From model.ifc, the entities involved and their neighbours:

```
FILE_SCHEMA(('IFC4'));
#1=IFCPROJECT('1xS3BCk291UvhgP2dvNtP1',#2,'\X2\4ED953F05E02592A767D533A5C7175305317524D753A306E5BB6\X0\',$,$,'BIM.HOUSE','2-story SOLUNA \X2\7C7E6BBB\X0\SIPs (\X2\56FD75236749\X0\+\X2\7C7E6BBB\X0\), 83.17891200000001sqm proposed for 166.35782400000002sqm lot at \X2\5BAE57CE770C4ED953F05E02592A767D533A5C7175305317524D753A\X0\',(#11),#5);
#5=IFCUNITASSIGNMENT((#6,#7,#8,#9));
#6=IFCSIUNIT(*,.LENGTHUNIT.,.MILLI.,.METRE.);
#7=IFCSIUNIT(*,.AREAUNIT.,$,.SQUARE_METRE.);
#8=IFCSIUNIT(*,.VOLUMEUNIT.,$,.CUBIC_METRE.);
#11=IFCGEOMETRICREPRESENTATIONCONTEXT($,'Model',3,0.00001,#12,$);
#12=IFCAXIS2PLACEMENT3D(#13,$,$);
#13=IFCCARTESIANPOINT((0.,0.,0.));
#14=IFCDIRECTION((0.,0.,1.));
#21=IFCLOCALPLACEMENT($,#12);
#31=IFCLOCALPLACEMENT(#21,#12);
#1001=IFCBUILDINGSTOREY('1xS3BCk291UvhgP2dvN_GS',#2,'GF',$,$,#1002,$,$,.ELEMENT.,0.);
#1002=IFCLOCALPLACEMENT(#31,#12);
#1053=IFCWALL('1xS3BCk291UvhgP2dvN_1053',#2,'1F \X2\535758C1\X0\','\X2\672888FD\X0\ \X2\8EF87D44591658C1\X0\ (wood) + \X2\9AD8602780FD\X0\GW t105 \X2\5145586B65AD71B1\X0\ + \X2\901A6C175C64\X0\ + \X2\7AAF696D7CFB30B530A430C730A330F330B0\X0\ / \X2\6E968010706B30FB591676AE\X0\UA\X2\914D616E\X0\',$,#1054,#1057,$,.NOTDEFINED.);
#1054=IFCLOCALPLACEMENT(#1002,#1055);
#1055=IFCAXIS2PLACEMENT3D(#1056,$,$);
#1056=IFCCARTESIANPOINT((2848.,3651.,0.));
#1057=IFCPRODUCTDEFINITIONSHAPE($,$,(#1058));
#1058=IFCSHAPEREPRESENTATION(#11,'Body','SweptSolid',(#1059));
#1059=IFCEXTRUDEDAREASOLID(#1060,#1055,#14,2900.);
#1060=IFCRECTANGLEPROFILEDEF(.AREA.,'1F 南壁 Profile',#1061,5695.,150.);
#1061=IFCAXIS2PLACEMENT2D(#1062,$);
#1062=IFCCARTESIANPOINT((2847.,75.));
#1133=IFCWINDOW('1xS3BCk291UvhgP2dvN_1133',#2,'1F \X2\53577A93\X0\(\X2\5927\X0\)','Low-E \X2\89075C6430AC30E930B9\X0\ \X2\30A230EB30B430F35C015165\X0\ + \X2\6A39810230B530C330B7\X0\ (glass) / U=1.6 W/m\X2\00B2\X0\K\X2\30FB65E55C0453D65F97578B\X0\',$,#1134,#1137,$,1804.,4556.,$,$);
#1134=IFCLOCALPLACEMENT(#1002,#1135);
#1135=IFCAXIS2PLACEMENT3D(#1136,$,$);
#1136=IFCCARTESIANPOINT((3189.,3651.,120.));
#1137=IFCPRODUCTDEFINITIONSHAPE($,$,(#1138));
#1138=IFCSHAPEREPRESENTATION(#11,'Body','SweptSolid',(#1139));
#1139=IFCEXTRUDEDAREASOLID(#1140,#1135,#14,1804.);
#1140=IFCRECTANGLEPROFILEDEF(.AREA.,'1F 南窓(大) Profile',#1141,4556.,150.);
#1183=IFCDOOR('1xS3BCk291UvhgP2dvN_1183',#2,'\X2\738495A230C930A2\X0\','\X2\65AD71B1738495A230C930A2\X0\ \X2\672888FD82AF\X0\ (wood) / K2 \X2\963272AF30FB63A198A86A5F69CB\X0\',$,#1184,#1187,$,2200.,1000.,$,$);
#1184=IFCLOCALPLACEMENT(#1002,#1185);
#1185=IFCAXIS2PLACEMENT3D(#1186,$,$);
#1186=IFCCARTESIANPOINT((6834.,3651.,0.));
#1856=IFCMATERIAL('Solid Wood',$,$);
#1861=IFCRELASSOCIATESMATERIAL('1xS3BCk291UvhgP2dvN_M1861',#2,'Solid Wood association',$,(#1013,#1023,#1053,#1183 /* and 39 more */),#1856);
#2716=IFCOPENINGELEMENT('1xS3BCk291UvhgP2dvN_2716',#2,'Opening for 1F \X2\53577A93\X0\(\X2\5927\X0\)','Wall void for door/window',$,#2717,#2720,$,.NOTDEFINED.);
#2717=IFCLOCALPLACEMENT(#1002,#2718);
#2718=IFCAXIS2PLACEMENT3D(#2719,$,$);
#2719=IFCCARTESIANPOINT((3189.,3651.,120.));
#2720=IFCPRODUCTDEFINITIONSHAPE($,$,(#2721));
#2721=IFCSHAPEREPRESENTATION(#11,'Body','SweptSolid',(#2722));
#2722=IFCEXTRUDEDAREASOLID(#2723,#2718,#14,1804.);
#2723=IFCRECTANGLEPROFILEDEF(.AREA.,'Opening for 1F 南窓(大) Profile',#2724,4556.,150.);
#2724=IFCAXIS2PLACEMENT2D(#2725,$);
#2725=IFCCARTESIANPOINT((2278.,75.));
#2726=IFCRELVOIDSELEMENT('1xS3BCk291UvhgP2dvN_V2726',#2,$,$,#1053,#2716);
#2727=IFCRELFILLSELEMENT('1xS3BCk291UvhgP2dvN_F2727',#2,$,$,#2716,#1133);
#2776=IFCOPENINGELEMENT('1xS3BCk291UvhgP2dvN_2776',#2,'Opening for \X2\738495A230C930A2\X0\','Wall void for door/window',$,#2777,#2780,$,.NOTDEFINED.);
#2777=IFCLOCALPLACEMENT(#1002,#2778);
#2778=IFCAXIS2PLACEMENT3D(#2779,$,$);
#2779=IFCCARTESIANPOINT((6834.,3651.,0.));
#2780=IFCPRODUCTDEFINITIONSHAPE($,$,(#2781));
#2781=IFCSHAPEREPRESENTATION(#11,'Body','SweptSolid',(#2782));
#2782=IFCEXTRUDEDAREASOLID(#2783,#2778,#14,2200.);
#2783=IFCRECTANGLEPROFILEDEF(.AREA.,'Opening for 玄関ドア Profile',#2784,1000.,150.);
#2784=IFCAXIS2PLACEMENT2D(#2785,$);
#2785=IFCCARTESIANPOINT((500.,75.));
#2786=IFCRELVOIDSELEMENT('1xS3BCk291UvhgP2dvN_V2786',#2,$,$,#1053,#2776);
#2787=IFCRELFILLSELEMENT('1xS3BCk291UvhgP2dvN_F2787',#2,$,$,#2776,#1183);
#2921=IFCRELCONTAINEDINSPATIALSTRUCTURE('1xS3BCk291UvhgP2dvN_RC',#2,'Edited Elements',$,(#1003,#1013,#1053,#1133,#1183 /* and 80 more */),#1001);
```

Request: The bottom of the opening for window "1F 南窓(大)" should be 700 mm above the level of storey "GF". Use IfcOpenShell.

```python
import numpy as np
import ifcopenshell
import ifcopenshell.api.geometry
import ifcopenshell.geom
import ifcopenshell.util.element
import ifcopenshell.util.placement
import ifcopenshell.util.shape
import ifcopenshell.util.unit

model = ifcopenshell.open("model.ifc")
unit_scale = ifcopenshell.util.unit.calculate_unit_scale(model)

window = model.by_id(1133)
opening = window.FillsVoids[0].RelatingOpeningElement
storey = ifcopenshell.util.element.get_container(window, ifc_class="IfcBuildingStorey")
level = ifcopenshell.util.placement.get_local_placement(storey.ObjectPlacement)[2, 3]

# The opening's origin need not be at the sill, so measure its lowest point.
shape = ifcopenshell.geom.create_shape(ifcopenshell.geom.settings(), opening)
bottom = ifcopenshell.util.shape.get_shape_bottom_elevation(shape, shape.geometry) / unit_scale
dz = level + 700.0 - bottom

shift = np.array([0.0, 0.0, dz])
# The window is not placed relative to its opening, so move both.
for product in (opening, window):
    matrix = ifcopenshell.util.placement.get_local_placement(product.ObjectPlacement)
    matrix[:3, 3] += shift
    ifcopenshell.api.geometry.edit_object_placement(model, product=product, matrix=matrix, is_si=False)

print(f"moved by {dz * unit_scale:+.3f} m")

model.write("model-out.ifc")
```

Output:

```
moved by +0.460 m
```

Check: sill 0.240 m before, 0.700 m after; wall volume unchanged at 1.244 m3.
